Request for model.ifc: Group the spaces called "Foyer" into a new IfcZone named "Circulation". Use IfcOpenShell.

First a look at what the model holds.

```python
import ifcopenshell

model = ifcopenshell.open("model.ifc")
print(model.schema)
seen = {}
for space in model.by_type("IfcSpace"):
    seen[space.LongName] = seen.get(space.LongName, 0) + 1
for name, count in sorted(seen.items(), key=str):
    print(count, "x", name)
print("zones:", [z.Name for z in model.by_type("IfcZone")][:20])
```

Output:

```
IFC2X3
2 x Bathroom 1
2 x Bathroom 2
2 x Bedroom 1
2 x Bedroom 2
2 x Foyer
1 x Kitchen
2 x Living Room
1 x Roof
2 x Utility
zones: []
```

```python
import ifcopenshell
import ifcopenshell.api.group
import ifcopenshell.api.root

model = ifcopenshell.open("model.ifc")

names = {"Foyer"}
spaces = [s for s in model.by_type("IfcSpace") if s.LongName in names]

zone = ifcopenshell.api.root.create_entity(model, ifc_class="IfcZone", name="Circulation")
ifcopenshell.api.group.assign_group(model, products=spaces, group=zone)
print(len(spaces), "spaces in", zone.Name)

model.write("model-out.ifc")
```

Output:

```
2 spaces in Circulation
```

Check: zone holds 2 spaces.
